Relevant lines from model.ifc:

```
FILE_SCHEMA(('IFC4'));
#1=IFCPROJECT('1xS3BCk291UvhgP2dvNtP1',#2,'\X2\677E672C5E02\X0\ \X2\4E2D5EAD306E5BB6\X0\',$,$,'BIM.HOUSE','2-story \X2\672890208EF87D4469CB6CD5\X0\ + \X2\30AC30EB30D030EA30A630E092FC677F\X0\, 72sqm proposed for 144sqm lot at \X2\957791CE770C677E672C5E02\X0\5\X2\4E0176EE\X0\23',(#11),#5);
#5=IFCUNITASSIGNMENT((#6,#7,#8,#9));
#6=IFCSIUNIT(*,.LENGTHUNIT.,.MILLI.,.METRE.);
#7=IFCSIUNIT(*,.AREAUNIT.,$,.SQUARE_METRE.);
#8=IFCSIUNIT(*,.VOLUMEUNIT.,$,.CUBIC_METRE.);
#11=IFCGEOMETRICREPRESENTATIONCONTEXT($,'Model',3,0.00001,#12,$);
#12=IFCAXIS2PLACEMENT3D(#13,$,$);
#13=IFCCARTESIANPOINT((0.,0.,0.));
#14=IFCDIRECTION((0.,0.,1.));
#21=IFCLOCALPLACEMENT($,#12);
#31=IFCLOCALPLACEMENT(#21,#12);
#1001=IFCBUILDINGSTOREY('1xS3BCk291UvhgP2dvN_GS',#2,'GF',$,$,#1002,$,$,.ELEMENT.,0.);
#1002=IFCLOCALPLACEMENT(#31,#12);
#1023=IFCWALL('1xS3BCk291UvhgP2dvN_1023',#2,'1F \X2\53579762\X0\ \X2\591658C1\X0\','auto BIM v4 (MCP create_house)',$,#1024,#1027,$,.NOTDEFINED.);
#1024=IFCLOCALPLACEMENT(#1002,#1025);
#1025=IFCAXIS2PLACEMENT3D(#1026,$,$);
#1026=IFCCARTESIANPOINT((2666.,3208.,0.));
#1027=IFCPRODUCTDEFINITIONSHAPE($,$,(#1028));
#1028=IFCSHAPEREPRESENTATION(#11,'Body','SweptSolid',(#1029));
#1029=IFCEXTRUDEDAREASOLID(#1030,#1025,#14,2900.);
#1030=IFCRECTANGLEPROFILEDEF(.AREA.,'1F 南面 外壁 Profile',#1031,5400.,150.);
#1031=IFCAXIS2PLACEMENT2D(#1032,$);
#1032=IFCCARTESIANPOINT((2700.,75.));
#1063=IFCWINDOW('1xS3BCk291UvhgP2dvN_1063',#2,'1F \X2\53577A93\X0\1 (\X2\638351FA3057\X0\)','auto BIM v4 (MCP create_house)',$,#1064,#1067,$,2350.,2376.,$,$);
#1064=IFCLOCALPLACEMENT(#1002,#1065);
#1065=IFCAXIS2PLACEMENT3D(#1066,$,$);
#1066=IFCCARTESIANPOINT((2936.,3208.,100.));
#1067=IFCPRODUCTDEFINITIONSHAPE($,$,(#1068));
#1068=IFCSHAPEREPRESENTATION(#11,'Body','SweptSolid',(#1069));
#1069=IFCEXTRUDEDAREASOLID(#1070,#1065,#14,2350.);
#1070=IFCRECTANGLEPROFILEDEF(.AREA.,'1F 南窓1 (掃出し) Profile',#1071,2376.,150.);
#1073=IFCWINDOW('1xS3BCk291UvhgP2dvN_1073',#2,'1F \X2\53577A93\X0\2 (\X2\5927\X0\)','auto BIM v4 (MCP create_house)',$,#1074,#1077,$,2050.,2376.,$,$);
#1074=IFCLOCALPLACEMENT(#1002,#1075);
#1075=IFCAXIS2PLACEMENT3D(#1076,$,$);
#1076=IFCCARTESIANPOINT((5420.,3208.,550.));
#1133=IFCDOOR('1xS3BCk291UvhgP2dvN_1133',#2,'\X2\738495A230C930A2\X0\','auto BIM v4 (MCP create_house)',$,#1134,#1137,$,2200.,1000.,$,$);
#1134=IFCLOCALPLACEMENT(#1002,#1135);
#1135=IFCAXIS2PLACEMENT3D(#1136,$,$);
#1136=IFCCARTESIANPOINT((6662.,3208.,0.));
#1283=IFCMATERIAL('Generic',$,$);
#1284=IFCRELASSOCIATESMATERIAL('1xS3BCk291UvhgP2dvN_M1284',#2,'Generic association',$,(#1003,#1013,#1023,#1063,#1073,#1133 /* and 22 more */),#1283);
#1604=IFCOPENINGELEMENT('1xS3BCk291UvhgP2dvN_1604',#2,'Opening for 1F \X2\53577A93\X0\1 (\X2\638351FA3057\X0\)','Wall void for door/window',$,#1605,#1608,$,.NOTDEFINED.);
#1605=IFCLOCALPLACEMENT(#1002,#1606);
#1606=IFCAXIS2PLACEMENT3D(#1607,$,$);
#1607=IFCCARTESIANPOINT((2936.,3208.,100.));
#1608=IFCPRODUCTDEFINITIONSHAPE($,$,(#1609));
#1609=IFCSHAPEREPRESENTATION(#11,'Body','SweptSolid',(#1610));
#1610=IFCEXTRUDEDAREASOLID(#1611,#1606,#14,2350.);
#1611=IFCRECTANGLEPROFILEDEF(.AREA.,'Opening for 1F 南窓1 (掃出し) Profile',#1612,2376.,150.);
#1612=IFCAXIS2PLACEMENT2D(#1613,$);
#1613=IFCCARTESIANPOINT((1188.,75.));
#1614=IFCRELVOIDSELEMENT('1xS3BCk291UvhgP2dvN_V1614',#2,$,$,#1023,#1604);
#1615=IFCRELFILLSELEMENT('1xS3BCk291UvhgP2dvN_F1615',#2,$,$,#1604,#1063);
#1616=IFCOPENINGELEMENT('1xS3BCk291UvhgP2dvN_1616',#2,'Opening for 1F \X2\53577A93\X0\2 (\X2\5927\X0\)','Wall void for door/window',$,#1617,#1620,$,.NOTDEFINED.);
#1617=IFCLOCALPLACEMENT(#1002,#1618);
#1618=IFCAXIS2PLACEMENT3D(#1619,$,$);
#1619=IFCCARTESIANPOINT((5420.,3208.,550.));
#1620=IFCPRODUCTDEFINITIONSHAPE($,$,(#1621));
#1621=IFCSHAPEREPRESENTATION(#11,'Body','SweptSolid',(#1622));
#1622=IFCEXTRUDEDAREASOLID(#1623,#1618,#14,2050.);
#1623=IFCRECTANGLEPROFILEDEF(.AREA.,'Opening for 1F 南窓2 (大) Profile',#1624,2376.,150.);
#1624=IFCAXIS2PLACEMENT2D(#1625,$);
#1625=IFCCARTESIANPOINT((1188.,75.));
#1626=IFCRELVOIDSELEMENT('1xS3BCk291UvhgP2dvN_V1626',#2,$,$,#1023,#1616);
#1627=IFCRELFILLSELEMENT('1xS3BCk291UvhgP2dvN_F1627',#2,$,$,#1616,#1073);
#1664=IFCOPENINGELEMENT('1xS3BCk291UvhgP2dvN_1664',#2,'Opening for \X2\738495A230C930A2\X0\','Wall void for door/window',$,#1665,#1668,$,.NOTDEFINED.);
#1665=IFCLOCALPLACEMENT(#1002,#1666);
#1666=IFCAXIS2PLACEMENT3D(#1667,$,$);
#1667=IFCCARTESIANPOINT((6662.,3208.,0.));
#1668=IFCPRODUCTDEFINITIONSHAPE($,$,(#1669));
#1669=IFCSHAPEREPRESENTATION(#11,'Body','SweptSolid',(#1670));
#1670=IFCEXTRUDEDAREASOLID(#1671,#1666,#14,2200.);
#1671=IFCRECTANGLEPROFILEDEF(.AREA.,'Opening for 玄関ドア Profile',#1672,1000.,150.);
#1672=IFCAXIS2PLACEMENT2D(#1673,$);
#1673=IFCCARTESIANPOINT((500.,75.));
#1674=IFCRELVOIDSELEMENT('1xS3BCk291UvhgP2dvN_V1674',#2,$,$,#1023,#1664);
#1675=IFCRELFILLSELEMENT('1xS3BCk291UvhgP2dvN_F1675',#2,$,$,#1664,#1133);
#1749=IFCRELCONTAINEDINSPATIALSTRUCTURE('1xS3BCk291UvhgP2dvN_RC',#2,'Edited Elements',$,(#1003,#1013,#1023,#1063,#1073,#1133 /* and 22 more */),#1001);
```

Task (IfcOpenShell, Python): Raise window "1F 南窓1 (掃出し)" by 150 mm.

```python
import numpy as np
import ifcopenshell
import ifcopenshell.api.geometry
import ifcopenshell.util.placement
import ifcopenshell.util.unit

model = ifcopenshell.open("model.ifc")
unit_scale = ifcopenshell.util.unit.calculate_unit_scale(model)

window = model.by_id(1063)
opening = window.FillsVoids[0].RelatingOpeningElement
dz = 0.15 / unit_scale

shift = np.array([0.0, 0.0, dz])
# The window is not placed relative to its opening, so move both.
for product in (opening, window):
    matrix = ifcopenshell.util.placement.get_local_placement(product.ObjectPlacement)
    matrix[:3, 3] += shift
    ifcopenshell.api.geometry.edit_object_placement(model, product=product, matrix=matrix, is_si=False)

print(f"moved by {dz * unit_scale:+.3f} m")

model.write("model_updated.ifc")
```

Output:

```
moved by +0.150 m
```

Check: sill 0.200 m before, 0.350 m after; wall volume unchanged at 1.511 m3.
